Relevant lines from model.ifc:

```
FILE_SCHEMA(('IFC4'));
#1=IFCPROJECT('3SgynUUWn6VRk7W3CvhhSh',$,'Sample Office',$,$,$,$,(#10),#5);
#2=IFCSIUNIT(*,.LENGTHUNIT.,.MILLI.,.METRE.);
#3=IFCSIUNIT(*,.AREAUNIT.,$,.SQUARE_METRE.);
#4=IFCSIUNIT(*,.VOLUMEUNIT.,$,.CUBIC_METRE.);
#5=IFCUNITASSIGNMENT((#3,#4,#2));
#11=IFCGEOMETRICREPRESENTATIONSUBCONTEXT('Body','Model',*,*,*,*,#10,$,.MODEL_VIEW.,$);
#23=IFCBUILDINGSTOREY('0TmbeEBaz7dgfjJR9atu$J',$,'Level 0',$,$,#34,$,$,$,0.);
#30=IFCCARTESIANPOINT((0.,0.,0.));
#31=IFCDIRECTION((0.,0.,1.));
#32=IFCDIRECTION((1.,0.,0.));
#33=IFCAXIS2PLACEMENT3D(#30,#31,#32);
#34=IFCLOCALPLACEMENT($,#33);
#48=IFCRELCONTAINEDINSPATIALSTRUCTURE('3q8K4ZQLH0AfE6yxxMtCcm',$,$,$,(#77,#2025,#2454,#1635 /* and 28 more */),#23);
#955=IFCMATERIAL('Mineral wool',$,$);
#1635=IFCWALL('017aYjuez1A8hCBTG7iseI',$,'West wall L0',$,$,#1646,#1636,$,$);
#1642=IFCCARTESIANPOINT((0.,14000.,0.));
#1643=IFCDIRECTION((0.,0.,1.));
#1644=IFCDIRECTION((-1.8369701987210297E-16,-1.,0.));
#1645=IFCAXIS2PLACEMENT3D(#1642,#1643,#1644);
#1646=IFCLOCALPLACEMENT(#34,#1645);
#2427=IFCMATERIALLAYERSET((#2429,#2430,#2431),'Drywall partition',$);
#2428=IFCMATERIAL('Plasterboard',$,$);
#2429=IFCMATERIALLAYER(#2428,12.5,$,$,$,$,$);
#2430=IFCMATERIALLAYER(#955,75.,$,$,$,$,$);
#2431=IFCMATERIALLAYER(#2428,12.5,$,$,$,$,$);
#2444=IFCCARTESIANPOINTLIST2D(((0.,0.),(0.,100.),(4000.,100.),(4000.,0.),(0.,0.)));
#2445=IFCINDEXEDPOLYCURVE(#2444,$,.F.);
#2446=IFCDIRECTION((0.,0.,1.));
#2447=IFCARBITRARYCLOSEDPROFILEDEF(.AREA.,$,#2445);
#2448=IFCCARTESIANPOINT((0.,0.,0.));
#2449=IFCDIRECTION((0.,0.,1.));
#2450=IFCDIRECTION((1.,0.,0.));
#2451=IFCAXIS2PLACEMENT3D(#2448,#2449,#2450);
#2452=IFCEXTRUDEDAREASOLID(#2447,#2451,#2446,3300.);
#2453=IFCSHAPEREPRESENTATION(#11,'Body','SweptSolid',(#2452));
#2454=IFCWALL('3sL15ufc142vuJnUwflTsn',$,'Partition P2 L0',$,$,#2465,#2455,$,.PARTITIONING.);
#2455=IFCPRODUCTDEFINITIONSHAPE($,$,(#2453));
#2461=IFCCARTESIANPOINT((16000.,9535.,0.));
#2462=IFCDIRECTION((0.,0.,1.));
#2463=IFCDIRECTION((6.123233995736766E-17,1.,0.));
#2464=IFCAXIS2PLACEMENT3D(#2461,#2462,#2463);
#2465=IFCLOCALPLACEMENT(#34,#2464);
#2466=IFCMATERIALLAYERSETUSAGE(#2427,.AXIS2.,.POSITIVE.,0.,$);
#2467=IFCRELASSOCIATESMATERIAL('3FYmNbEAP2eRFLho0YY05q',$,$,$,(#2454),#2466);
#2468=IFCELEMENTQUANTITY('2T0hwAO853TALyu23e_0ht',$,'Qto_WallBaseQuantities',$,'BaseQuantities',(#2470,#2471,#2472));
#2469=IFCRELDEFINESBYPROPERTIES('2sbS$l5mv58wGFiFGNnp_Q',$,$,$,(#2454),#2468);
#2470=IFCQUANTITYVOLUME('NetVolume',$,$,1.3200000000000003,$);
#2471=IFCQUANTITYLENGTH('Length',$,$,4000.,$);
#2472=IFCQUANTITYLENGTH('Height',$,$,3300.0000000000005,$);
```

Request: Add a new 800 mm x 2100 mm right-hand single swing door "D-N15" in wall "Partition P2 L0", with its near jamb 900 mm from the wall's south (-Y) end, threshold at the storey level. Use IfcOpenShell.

```python
import numpy as np
import ifcopenshell
import ifcopenshell.api.feature
import ifcopenshell.api.geometry
import ifcopenshell.api.pset
import ifcopenshell.api.root
import ifcopenshell.api.spatial
import ifcopenshell.geom
import ifcopenshell.util.element
import ifcopenshell.util.placement
import ifcopenshell.util.representation
import ifcopenshell.util.shape
import ifcopenshell.util.unit

model = ifcopenshell.open("model.ifc")
unit_scale = ifcopenshell.util.unit.calculate_unit_scale(model)
volume_scale = ifcopenshell.util.unit.calculate_unit_scale(model, "VOLUMEUNIT")
settings = ifcopenshell.geom.settings()


def volume(element):
    """Net volume in cubic metres, openings subtracted."""
    shape = ifcopenshell.geom.create_shape(settings, element)
    return ifcopenshell.util.shape.get_volume(shape.geometry)


wall = model.by_id(2454)
storey = ifcopenshell.util.element.get_container(wall, ifc_class="IfcBuildingStorey")
context = ifcopenshell.util.representation.get_context(model, "Model", "Body", "MODEL_VIEW")
before = volume(wall)

width, height, from_end, sill = 0.8, 2.1, 0.9, 0.0  # metres

# The wall runs along its own X axis, and the end named is its -X end.
wall_shape = ifcopenshell.geom.create_shape(settings, wall)
x, y, z = ifcopenshell.util.shape.get_vertices(wall_shape.geometry).T
start = x.min() + from_end
face, thickness = float(y.min()), float(y.max() - y.min())
wall_matrix = ifcopenshell.util.placement.get_local_placement(wall.ObjectPlacement)
level = ifcopenshell.util.placement.get_local_placement(storey.ObjectPlacement)[2, 3]


def in_wall(x, y):
    """Placement at x, y metres in the wall's axes, at sill height."""
    matrix = wall_matrix.copy()
    matrix[:, 3] = wall_matrix @ np.array([x / unit_scale, y / unit_scale, 0.0, 1.0])
    matrix[2, 3] = level + sill / unit_scale
    return matrix


# Opening: a box that overshoots both wall faces by 50 mm.
opening = ifcopenshell.api.root.create_entity(model, ifc_class="IfcOpeningElement", predefined_type="OPENING")
box = ifcopenshell.api.geometry.add_wall_representation(
    model, context=context, length=width, height=height, thickness=thickness + 0.1
)
ifcopenshell.api.geometry.assign_representation(model, product=opening, representation=box)
ifcopenshell.api.geometry.edit_object_placement(model, product=opening, matrix=in_wall(start, face - 0.05), is_si=False)
ifcopenshell.api.feature.add_feature(model, feature=opening, element=wall)

door = ifcopenshell.api.root.create_entity(model, ifc_class="IfcDoor", name="D-N15", predefined_type="DOOR")
door.OverallWidth, door.OverallHeight = width / unit_scale, height / unit_scale
door.OperationType = "SINGLE_SWING_RIGHT"
body = ifcopenshell.api.geometry.add_door_representation(
    model,
    context=context,
    overall_width=door.OverallWidth,
    overall_height=door.OverallHeight,
    operation_type="SINGLE_SWING_RIGHT",
    lining_properties={"LiningDepth": thickness / unit_scale, "ThresholdDepth": thickness / unit_scale},
)
ifcopenshell.api.geometry.assign_representation(model, product=door, representation=body)
ifcopenshell.api.spatial.assign_container(model, products=[door], relating_structure=storey)
ifcopenshell.api.feature.add_filling(model, opening=opening, element=door)

# The lining spans the wall, so the door starts at the wall face.
ifcopenshell.api.geometry.edit_object_placement(model, product=door, matrix=in_wall(start, face), is_si=False)

after = volume(wall)

# Update the wall's stored quantities.
qto = model.by_id(ifcopenshell.util.element.get_pset(wall, "Qto_WallBaseQuantities", should_inherit=False)["id"])
ifcopenshell.api.pset.edit_qto(model, qto=qto, properties={"NetVolume": after / volume_scale})

print(f"wall volume {before:.3f} -> {after:.3f} m3")

model.write("model_edited.ifc")
```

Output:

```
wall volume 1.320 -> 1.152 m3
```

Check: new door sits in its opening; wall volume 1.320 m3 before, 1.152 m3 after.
